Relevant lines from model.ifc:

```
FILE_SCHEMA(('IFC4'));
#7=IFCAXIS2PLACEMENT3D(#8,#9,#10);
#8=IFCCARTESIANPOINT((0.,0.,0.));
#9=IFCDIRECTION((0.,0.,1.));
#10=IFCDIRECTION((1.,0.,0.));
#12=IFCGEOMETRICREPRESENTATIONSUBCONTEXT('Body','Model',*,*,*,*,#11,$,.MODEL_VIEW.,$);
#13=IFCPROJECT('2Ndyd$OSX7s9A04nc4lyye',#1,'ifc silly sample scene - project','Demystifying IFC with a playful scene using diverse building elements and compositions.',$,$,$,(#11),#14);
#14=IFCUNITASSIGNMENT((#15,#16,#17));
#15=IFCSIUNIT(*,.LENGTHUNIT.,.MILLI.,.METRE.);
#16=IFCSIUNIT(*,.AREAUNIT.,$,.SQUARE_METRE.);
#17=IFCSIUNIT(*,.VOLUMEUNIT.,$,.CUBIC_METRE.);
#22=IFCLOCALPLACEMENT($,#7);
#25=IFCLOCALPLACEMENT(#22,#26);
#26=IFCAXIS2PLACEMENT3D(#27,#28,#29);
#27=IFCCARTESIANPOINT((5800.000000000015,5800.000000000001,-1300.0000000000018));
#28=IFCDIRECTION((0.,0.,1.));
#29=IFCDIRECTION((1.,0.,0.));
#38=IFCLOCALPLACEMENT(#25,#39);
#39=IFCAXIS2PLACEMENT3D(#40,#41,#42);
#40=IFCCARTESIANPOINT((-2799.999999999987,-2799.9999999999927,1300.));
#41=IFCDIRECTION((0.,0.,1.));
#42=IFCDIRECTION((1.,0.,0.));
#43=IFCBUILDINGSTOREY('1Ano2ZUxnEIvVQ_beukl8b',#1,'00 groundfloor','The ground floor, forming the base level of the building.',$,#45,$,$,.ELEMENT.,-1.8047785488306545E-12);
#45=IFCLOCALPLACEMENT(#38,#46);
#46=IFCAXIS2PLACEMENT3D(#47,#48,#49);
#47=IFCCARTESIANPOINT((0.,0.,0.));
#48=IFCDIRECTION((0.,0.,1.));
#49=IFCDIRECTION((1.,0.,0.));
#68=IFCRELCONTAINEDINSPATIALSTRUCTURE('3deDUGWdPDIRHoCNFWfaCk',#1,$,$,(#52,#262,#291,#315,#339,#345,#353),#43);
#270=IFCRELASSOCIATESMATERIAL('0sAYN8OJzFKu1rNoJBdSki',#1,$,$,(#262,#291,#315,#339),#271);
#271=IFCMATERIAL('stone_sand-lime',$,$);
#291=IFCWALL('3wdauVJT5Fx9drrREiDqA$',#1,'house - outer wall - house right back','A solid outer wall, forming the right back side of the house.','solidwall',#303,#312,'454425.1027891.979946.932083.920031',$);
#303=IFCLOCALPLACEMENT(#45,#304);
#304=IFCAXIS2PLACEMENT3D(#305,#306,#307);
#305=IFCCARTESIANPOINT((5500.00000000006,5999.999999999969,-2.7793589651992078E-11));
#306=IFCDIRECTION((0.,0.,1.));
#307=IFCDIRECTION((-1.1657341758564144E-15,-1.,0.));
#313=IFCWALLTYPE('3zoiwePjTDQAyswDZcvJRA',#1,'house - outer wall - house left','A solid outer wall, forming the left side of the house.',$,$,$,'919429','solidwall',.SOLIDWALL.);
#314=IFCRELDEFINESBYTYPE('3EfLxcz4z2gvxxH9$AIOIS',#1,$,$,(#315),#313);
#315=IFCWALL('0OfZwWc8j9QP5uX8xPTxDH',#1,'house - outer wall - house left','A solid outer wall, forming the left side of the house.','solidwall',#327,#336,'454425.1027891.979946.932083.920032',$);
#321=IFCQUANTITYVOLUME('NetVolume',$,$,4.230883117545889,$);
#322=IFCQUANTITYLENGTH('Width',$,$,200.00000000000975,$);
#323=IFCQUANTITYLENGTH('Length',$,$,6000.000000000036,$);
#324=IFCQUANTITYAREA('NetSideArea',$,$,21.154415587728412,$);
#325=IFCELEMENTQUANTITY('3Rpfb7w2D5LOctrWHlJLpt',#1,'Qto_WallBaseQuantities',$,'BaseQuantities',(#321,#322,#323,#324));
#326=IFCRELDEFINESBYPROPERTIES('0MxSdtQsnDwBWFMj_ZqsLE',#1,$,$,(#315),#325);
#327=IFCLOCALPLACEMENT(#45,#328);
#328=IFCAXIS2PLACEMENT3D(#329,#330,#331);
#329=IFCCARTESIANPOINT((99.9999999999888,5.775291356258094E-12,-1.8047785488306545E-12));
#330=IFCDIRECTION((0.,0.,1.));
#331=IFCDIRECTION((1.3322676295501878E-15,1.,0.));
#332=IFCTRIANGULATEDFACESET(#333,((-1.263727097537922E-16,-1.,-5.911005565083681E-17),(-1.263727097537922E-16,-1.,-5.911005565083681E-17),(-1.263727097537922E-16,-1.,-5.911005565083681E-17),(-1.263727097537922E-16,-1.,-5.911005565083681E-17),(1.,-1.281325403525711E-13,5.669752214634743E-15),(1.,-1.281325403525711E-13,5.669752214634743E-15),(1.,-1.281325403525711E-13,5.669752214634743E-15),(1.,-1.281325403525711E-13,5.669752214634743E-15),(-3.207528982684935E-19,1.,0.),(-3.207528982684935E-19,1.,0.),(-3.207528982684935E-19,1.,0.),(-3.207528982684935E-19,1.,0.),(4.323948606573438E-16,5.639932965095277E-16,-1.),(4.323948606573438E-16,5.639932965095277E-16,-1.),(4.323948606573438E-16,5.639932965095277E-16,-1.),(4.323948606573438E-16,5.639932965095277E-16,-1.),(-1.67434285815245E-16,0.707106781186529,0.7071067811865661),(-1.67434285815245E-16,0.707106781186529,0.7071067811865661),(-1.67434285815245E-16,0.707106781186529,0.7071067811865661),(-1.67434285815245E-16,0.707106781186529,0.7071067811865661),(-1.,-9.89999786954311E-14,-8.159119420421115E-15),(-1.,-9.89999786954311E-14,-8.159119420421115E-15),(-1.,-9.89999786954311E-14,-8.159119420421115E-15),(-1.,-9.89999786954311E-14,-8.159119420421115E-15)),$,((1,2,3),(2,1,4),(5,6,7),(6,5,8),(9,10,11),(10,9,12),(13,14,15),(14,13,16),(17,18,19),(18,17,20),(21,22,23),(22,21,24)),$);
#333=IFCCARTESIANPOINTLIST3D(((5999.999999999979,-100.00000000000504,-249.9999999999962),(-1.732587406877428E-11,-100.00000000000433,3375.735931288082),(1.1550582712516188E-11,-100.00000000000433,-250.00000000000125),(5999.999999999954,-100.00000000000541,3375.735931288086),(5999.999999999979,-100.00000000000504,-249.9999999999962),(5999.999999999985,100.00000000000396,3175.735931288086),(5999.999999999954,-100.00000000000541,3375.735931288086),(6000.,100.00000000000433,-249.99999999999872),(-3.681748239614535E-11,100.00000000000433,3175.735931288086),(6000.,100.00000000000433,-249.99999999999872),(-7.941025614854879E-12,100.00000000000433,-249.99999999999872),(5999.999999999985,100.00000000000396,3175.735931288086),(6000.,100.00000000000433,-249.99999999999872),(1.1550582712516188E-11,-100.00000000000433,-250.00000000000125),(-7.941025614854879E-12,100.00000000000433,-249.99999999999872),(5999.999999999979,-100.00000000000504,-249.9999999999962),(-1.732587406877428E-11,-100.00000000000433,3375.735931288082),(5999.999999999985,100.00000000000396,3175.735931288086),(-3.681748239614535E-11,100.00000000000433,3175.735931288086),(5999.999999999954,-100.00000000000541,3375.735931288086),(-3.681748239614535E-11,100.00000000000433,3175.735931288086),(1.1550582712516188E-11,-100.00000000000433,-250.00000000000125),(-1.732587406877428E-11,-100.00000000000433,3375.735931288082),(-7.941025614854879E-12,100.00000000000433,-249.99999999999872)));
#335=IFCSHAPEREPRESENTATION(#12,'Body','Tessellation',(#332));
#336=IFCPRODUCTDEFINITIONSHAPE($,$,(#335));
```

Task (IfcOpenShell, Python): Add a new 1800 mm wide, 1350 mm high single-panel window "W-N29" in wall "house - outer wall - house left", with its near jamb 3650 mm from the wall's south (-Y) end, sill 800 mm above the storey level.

```python
import numpy as np
import ifcopenshell
import ifcopenshell.api.feature
import ifcopenshell.api.geometry
import ifcopenshell.api.pset
import ifcopenshell.api.root
import ifcopenshell.api.spatial
import ifcopenshell.geom
import ifcopenshell.util.element
import ifcopenshell.util.placement
import ifcopenshell.util.representation
import ifcopenshell.util.shape
import ifcopenshell.util.unit

model = ifcopenshell.open("model.ifc")
unit_scale = ifcopenshell.util.unit.calculate_unit_scale(model)
area_scale = ifcopenshell.util.unit.calculate_unit_scale(model, "AREAUNIT")
volume_scale = ifcopenshell.util.unit.calculate_unit_scale(model, "VOLUMEUNIT")
settings = ifcopenshell.geom.settings()


def volume(element):
    """Net volume in cubic metres, openings subtracted."""
    shape = ifcopenshell.geom.create_shape(settings, element)
    return ifcopenshell.util.shape.get_volume(shape.geometry)


wall = model.by_guid("0OfZwWc8j9QP5uX8xPTxDH")
storey = ifcopenshell.util.element.get_container(wall, ifc_class="IfcBuildingStorey")
context = ifcopenshell.util.representation.get_context(model, "Model", "Body", "MODEL_VIEW")
before = volume(wall)

width, height, from_end, sill = 1.8, 1.35, 3.65, 0.8  # metres

# The wall runs along its own X axis, and the end named is its -X end.
wall_shape = ifcopenshell.geom.create_shape(settings, wall)
x, y, z = ifcopenshell.util.shape.get_vertices(wall_shape.geometry).T
start = x.min() + from_end
face, thickness = float(y.min()), float(y.max() - y.min())
wall_matrix = ifcopenshell.util.placement.get_local_placement(wall.ObjectPlacement)
level = ifcopenshell.util.placement.get_local_placement(storey.ObjectPlacement)[2, 3]


def in_wall(x, y):
    """Placement at x, y metres in the wall's axes, at sill height."""
    matrix = wall_matrix.copy()
    matrix[:, 3] = wall_matrix @ np.array([x / unit_scale, y / unit_scale, 0.0, 1.0])
    matrix[2, 3] = level + sill / unit_scale
    return matrix


# Opening: a box that overshoots both wall faces by 50 mm.
opening = ifcopenshell.api.root.create_entity(model, ifc_class="IfcOpeningElement", predefined_type="OPENING")
box = ifcopenshell.api.geometry.add_wall_representation(
    model, context=context, length=width, height=height, thickness=thickness + 0.1
)
ifcopenshell.api.geometry.assign_representation(model, product=opening, representation=box)
ifcopenshell.api.geometry.edit_object_placement(model, product=opening, matrix=in_wall(start, face - 0.05), is_si=False)
ifcopenshell.api.feature.add_feature(model, feature=opening, element=wall)

window = ifcopenshell.api.root.create_entity(model, ifc_class="IfcWindow", name="W-N29", predefined_type="WINDOW")
window.OverallWidth, window.OverallHeight = width / unit_scale, height / unit_scale
window.PartitioningType = "SINGLE_PANEL"
body = ifcopenshell.api.geometry.add_window_representation(
    model,
    context=context,
    overall_width=window.OverallWidth,
    overall_height=window.OverallHeight,
    partition_type="SINGLE_PANEL",
)
ifcopenshell.api.geometry.assign_representation(model, product=window, representation=body)
ifcopenshell.api.spatial.assign_container(model, products=[window], relating_structure=storey)
ifcopenshell.api.feature.add_filling(model, opening=opening, element=window)

# Centre the window in the wall's thickness.
ifcopenshell.api.geometry.edit_object_placement(model, product=window, matrix=in_wall(start, face), is_si=False)
window_shape = ifcopenshell.geom.create_shape(settings, window)
depth = ifcopenshell.util.shape.get_vertices(window_shape.geometry)[:, 1]
offset = face + thickness / 2 - (depth.min() + depth.max()) / 2
ifcopenshell.api.geometry.edit_object_placement(model, product=window, matrix=in_wall(start, offset), is_si=False)

after = volume(wall)

# Update the wall's stored quantities.
qto = model.by_id(ifcopenshell.util.element.get_pset(wall, "Qto_WallBaseQuantities", should_inherit=False)["id"])
ifcopenshell.api.pset.edit_qto(model, qto=qto, properties={
    "NetVolume": after / volume_scale,
    "NetSideArea": after / thickness / area_scale,
})

print(f"wall volume {before:.3f} -> {after:.3f} m3")

model.write("model_v2.ifc")
```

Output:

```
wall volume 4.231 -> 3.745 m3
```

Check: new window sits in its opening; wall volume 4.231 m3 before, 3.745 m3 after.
